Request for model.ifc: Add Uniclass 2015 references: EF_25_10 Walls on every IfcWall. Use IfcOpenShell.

First a look at what the model holds.

```python
import ifcopenshell

model = ifcopenshell.open("model.ifc")
print(model.schema)
print("classifications:", [c.Name for c in model.by_type("IfcClassification")])
for ifc_class in ("IfcDoor", "IfcRoof", "IfcStair", "IfcWall", "IfcWindow"):
    print(ifc_class, len(model.by_type(ifc_class)))
```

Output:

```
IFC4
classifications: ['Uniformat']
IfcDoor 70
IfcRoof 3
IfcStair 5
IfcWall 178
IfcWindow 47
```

```python
import ifcopenshell
import ifcopenshell.api.classification

model = ifcopenshell.open("model.ifc")

system = ifcopenshell.api.classification.add_classification(model, classification="Uniclass 2015")

codes = {
    "IfcWall": ("EF_25_10", "Walls"),
}
for ifc_class, (code, name) in codes.items():
    products = model.by_type(ifc_class)
    ifcopenshell.api.classification.add_reference(
        model, products=products, classification=system, identification=code, name=name
    )
    print(code, len(products))

model.write("model-out.ifc")
```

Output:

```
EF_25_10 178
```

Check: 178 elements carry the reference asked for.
